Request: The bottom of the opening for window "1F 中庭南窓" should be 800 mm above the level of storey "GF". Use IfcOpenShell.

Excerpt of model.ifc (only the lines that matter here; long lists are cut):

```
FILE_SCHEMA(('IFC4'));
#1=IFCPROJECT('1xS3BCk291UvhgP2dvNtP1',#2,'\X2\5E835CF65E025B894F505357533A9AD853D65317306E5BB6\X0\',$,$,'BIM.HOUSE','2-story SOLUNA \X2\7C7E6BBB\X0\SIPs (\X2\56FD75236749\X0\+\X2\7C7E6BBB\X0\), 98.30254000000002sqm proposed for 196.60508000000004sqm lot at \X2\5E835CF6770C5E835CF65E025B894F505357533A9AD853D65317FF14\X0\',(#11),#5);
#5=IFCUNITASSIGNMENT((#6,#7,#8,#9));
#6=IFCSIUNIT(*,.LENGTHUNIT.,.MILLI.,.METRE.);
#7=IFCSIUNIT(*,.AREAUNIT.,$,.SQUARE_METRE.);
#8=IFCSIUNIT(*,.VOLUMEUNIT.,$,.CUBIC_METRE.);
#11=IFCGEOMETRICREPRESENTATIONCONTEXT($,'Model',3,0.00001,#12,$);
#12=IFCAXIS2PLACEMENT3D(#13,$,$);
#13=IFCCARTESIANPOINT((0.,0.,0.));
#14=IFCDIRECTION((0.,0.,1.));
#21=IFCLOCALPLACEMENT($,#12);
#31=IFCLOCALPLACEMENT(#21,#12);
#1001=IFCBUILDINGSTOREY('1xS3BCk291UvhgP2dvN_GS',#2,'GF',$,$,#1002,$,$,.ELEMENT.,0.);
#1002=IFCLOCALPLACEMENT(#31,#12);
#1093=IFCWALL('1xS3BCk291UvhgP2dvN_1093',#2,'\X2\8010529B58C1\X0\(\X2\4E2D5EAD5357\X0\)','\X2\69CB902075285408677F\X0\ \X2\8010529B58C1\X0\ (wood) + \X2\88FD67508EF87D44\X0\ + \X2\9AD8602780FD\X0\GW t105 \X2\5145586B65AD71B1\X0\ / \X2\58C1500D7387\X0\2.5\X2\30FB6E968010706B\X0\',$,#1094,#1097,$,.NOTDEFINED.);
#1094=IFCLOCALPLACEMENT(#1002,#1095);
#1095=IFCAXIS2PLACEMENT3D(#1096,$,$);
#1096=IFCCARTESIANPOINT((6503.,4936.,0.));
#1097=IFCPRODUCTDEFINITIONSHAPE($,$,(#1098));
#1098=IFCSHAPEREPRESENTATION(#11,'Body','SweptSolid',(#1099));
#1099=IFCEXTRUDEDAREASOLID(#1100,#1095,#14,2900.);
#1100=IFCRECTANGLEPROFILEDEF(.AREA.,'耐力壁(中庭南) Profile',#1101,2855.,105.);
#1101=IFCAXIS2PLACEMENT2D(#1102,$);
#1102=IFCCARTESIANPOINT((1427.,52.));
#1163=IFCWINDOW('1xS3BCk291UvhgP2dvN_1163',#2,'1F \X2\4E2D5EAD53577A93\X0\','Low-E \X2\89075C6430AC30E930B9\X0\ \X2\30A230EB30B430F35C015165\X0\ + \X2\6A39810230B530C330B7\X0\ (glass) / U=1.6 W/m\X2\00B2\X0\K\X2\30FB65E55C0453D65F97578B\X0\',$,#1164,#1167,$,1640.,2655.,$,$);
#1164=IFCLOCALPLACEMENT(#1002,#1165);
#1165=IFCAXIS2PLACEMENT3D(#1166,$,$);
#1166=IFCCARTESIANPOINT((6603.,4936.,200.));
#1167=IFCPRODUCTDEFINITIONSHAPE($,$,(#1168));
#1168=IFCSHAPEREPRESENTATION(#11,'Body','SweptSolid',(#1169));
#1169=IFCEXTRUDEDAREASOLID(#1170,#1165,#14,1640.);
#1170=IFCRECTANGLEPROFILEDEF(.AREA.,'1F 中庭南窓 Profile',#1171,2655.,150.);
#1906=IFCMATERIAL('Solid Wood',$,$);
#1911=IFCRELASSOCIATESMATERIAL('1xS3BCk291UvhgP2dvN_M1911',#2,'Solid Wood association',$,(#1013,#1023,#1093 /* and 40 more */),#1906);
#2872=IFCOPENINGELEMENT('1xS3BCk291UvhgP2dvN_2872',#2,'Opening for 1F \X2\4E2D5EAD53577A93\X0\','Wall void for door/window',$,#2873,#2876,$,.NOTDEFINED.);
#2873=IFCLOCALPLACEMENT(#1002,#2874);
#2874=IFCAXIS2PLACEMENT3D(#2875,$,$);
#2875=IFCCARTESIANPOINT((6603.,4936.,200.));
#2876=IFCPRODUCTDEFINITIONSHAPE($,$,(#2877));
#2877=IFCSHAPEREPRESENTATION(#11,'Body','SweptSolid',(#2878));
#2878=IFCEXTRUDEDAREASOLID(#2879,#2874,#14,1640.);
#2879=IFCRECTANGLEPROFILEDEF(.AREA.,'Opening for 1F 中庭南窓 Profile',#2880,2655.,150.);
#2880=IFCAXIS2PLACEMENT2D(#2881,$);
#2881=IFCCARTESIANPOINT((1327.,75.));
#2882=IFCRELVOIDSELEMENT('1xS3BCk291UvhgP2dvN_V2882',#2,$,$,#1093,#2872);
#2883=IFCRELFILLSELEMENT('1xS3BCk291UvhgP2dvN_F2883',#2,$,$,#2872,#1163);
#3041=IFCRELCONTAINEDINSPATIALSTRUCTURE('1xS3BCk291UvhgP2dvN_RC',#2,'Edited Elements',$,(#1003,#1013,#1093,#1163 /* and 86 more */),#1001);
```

```python
import numpy as np
import ifcopenshell
import ifcopenshell.api.geometry
import ifcopenshell.geom
import ifcopenshell.util.element
import ifcopenshell.util.placement
import ifcopenshell.util.shape
import ifcopenshell.util.unit

model = ifcopenshell.open("model.ifc")
unit_scale = ifcopenshell.util.unit.calculate_unit_scale(model)

window = model.by_guid("1xS3BCk291UvhgP2dvN_1163")
opening = window.FillsVoids[0].RelatingOpeningElement
storey = ifcopenshell.util.element.get_container(window, ifc_class="IfcBuildingStorey")
level = ifcopenshell.util.placement.get_local_placement(storey.ObjectPlacement)[2, 3]

# The opening's origin need not be at the sill, so measure its lowest point.
shape = ifcopenshell.geom.create_shape(ifcopenshell.geom.settings(), opening)
bottom = ifcopenshell.util.shape.get_shape_bottom_elevation(shape, shape.geometry) / unit_scale
dz = level + 0.8 / unit_scale - bottom

shift = np.array([0.0, 0.0, dz])
# The window is not placed relative to its opening, so move both.
for product in (opening, window):
    matrix = ifcopenshell.util.placement.get_local_placement(product.ObjectPlacement)
    matrix[:3, 3] += shift
    ifcopenshell.api.geometry.edit_object_placement(model, product=product, matrix=matrix, is_si=False)

print(f"moved by {dz * unit_scale:+.3f} m")

model.write("model_rev.ifc")
```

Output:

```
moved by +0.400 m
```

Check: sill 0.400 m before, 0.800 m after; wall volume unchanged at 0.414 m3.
